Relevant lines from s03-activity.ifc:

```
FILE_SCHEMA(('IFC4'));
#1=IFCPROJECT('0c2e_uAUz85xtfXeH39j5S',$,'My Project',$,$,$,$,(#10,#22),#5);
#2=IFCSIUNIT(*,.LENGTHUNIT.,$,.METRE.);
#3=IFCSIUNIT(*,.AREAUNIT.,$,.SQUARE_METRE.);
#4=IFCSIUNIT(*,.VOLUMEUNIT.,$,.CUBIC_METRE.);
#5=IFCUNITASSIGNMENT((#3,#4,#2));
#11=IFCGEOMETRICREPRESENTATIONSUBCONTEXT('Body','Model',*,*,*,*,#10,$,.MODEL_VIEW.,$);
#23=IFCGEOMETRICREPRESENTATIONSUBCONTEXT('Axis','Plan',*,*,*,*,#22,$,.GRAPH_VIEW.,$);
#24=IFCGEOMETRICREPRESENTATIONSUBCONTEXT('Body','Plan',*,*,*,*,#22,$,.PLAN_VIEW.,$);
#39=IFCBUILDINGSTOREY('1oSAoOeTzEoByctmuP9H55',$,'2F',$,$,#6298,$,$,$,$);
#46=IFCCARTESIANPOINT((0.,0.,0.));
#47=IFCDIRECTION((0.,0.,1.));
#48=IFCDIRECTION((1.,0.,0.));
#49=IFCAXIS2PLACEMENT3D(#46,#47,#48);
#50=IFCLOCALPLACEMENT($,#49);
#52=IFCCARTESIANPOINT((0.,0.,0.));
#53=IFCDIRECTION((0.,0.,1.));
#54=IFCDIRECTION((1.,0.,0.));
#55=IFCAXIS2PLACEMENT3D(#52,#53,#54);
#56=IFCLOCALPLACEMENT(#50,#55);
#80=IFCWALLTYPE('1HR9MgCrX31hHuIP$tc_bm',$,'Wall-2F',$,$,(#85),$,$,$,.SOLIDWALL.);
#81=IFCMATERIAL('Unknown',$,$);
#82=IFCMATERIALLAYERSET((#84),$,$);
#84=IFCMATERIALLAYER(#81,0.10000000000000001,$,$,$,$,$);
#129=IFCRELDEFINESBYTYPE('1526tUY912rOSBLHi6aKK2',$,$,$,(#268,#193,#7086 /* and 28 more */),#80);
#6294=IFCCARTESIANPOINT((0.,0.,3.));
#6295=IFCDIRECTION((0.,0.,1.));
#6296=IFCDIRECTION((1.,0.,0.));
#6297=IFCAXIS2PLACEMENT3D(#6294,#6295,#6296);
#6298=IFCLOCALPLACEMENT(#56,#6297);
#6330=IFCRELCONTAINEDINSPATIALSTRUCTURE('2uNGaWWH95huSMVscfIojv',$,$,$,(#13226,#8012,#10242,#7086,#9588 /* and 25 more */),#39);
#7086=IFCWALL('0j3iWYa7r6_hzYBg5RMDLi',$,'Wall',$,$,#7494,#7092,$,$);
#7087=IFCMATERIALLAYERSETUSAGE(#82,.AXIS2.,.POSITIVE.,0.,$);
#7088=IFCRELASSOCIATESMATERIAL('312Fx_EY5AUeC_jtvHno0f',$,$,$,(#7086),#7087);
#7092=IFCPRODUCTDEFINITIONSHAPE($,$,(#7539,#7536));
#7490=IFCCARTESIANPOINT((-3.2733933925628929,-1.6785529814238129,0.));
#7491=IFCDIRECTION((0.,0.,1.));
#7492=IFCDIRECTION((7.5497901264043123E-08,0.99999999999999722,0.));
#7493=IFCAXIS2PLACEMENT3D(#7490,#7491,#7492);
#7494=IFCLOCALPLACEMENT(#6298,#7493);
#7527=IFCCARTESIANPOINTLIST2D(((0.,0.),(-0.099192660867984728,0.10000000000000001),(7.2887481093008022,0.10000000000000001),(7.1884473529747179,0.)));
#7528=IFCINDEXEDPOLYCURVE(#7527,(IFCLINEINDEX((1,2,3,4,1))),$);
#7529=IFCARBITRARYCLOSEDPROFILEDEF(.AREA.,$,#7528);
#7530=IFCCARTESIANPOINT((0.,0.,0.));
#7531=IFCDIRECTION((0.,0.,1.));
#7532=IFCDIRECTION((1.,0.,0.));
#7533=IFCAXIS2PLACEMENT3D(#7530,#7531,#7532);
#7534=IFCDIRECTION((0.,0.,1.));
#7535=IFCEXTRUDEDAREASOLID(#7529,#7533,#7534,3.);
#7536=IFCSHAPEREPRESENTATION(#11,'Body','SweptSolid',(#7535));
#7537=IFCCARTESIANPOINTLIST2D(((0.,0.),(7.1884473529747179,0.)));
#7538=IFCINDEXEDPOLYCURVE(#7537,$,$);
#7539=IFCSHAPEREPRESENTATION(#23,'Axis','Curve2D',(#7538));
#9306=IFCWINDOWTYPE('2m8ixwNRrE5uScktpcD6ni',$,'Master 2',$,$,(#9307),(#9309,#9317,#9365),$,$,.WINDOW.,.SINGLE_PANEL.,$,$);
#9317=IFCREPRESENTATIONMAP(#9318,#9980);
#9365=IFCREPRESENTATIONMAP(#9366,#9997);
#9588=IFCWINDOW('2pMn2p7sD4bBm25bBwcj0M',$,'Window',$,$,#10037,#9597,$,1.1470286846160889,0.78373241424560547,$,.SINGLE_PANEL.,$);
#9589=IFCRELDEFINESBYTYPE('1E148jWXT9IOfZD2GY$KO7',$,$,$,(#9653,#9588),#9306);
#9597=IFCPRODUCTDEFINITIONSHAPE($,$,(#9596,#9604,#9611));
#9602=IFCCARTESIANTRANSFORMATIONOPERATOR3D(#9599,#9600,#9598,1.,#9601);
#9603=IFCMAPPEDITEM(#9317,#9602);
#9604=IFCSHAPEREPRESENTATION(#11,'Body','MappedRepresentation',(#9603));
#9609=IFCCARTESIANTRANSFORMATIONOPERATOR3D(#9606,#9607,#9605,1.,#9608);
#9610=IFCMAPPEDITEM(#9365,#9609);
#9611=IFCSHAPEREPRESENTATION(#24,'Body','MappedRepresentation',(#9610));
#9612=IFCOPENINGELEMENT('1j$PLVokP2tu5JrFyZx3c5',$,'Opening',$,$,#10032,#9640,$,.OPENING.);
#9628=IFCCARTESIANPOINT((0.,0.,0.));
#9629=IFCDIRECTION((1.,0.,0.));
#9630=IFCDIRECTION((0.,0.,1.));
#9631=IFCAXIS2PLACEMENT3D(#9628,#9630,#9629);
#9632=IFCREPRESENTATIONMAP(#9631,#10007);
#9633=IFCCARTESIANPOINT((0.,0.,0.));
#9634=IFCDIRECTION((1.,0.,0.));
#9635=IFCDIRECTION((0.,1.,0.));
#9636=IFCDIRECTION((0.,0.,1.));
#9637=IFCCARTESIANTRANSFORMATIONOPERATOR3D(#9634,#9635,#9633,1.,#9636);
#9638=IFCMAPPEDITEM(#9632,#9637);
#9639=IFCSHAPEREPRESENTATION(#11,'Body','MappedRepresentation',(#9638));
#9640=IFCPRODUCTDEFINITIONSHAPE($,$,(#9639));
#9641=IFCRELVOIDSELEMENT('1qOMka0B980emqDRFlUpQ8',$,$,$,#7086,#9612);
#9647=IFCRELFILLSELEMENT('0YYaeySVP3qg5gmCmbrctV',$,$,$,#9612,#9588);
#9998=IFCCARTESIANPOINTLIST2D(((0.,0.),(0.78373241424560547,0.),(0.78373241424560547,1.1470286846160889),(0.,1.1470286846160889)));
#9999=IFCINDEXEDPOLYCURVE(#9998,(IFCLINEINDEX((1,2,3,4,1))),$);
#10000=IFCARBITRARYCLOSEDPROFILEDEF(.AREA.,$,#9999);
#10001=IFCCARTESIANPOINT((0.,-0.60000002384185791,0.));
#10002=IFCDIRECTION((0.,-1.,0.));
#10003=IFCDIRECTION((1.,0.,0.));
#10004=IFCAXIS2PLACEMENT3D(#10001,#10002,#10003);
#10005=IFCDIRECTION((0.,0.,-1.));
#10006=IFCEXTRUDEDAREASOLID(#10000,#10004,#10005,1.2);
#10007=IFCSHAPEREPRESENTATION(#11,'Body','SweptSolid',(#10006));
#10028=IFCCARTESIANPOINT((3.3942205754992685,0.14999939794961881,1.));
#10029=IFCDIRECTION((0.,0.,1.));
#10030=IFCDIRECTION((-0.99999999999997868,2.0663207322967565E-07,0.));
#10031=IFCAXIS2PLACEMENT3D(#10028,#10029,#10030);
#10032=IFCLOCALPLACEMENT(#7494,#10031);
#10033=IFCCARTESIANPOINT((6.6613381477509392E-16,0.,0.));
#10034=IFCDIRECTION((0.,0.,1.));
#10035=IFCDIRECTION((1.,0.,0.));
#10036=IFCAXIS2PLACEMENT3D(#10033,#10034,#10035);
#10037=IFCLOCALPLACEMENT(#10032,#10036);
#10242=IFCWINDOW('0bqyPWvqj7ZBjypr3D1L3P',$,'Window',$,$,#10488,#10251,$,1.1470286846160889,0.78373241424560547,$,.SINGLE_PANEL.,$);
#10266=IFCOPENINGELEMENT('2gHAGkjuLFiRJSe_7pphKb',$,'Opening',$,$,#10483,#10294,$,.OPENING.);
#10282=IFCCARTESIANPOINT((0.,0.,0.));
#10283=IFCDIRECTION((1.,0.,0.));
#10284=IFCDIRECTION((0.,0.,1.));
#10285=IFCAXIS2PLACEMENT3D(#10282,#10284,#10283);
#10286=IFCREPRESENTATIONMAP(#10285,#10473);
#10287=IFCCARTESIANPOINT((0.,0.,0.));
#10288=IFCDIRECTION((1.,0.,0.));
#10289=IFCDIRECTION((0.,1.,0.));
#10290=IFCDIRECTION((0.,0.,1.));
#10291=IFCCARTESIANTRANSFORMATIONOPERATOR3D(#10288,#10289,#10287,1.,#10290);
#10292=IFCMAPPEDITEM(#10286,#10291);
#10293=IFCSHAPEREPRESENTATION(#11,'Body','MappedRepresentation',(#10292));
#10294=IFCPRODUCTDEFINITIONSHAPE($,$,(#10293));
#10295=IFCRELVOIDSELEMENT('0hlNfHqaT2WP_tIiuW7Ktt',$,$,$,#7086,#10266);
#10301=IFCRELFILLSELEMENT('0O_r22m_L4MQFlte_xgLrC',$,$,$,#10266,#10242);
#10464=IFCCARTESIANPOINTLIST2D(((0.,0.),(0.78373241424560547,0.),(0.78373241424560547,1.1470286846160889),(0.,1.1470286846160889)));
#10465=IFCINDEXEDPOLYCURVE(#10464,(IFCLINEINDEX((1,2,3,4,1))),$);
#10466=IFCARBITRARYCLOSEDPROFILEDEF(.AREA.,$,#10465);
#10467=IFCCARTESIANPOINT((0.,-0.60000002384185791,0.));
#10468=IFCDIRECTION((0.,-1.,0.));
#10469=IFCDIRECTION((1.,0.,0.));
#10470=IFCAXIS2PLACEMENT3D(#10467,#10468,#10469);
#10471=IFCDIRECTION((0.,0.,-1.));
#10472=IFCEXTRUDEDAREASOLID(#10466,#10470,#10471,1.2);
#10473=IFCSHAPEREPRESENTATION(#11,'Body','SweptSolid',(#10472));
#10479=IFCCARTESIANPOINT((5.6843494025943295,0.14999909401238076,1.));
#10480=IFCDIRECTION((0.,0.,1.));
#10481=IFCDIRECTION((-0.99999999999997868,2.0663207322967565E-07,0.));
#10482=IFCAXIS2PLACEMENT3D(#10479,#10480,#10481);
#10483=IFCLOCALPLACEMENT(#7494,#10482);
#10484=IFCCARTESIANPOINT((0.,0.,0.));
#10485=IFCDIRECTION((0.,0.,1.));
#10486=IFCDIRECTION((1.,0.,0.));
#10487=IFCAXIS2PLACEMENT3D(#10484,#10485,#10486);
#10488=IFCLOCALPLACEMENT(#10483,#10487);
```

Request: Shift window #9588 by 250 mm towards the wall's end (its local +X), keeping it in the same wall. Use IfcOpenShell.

```python
import ifcopenshell
import ifcopenshell.api.geometry
import ifcopenshell.util.placement

model = ifcopenshell.open("s03-activity.ifc")

window = model.by_id(9588)
opening = window.FillsVoids[0].RelatingOpeningElement
wall = opening.VoidsElements[0].RelatingBuildingElement

wall_matrix = ifcopenshell.util.placement.get_local_placement(wall.ObjectPlacement)
shift = wall_matrix[:3, 0] * 0.25
before = ifcopenshell.util.placement.get_local_placement(window.ObjectPlacement)[:3, 3].copy()

# The window is placed relative to its opening, so it follows when the opening moves.
matrix = ifcopenshell.util.placement.get_local_placement(opening.ObjectPlacement)
matrix[:3, 3] += shift
ifcopenshell.api.geometry.edit_object_placement(
    model, product=opening, matrix=matrix, is_si=False, should_transform_children=True
)

after = ifcopenshell.util.placement.get_local_placement(window.ObjectPlacement)[:3, 3]
print("window moved by", (after - before).round(3) + 0.0)

model.write("s03-activity_updated.ifc")
```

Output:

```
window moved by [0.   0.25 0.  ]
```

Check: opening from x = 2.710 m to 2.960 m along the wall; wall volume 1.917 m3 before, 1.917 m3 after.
